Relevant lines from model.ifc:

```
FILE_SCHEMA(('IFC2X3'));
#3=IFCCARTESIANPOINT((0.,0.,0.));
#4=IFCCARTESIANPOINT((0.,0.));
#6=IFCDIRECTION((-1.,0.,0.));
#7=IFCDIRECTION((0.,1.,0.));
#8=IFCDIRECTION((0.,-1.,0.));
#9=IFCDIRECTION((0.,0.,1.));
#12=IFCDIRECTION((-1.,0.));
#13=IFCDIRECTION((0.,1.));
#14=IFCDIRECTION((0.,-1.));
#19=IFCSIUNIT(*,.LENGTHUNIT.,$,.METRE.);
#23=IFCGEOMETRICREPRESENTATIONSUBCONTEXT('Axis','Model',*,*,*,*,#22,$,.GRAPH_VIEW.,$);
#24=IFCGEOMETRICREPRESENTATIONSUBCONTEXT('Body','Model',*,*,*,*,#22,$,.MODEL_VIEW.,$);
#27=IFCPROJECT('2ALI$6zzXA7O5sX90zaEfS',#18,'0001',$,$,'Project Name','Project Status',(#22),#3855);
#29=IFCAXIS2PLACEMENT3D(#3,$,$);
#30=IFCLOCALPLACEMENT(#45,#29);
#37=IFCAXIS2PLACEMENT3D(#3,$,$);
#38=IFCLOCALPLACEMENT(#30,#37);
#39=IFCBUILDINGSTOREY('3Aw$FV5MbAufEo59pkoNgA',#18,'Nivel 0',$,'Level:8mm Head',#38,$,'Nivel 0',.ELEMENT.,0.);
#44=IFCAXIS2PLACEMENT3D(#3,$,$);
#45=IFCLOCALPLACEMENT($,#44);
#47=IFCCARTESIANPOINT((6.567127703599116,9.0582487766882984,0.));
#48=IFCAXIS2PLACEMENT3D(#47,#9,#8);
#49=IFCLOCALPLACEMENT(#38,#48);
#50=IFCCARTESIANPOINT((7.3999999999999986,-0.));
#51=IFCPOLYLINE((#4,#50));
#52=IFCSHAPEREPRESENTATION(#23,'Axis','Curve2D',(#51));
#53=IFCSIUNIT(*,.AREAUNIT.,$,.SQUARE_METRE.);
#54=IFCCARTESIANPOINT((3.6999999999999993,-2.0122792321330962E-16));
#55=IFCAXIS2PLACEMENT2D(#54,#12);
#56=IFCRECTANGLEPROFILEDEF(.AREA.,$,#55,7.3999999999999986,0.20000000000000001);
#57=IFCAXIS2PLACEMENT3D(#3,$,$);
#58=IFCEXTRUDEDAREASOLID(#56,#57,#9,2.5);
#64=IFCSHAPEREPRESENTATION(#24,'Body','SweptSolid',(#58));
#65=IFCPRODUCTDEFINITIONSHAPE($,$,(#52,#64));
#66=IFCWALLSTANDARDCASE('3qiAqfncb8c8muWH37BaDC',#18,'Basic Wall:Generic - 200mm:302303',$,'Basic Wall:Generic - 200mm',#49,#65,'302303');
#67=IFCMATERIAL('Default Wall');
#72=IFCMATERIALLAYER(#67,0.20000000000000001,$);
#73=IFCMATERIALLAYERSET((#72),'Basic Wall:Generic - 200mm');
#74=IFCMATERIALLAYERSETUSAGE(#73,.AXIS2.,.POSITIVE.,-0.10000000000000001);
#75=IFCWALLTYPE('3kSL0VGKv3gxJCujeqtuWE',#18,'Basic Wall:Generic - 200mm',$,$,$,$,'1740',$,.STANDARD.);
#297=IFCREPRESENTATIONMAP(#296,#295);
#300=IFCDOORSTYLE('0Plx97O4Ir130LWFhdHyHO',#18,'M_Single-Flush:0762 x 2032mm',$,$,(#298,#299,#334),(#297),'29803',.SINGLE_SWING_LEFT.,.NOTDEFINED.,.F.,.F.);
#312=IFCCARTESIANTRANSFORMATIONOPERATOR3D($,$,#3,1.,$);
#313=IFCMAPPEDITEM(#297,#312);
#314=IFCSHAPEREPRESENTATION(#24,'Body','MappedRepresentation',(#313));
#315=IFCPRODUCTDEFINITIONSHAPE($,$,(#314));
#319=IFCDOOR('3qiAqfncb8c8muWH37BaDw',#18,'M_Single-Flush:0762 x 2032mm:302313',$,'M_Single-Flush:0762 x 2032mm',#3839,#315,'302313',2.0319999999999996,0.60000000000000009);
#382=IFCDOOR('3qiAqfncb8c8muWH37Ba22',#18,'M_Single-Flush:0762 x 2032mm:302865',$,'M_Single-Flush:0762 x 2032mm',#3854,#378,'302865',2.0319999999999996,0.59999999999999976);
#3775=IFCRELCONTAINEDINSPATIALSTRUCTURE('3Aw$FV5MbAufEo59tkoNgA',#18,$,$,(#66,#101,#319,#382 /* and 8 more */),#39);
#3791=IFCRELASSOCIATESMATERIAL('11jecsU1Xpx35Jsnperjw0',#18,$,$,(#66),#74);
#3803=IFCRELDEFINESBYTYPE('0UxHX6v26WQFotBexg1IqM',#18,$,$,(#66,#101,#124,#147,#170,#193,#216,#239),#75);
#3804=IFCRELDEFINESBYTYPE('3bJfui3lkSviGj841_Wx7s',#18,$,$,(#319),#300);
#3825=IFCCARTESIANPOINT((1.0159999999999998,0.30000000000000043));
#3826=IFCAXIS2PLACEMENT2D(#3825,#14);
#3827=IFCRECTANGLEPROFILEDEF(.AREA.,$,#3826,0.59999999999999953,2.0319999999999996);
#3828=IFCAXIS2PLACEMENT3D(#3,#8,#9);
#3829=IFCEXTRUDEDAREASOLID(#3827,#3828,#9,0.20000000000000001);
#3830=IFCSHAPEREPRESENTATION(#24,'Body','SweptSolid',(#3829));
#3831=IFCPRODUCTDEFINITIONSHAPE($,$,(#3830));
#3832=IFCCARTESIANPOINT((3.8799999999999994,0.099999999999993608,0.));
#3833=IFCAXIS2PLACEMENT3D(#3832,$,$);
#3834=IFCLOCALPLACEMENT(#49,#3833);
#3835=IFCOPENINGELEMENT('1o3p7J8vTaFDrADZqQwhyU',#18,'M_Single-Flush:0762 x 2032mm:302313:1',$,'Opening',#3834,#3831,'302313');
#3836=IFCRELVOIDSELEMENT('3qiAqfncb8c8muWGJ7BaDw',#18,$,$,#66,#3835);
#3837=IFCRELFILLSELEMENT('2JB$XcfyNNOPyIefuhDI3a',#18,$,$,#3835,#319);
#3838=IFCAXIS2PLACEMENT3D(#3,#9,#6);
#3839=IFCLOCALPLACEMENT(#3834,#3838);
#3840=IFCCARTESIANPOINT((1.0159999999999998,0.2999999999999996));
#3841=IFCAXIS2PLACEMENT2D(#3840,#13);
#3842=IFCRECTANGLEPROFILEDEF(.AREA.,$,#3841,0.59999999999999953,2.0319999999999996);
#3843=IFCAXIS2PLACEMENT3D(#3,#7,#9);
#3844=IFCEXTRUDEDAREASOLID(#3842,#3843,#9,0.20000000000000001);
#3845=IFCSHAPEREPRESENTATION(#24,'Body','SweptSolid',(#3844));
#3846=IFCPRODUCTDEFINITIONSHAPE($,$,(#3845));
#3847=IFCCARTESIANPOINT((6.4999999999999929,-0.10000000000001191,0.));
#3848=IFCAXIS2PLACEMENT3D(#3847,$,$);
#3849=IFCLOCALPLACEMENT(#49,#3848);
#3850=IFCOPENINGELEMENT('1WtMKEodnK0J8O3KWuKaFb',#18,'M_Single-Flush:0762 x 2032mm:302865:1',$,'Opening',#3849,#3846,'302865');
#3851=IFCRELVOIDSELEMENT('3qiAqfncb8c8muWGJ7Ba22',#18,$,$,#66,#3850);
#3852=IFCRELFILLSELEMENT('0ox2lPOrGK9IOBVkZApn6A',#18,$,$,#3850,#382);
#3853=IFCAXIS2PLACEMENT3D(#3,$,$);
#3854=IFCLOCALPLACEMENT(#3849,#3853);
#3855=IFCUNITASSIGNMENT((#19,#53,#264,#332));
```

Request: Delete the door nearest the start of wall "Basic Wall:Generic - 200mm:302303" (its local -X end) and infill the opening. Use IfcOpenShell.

```python
import ifcopenshell
import ifcopenshell.api.feature
import ifcopenshell.api.root
import ifcopenshell.geom
import ifcopenshell.util.shape

model = ifcopenshell.open("model.ifc")
settings = ifcopenshell.geom.settings()


def volume(element):
    """Net volume in cubic metres, openings subtracted."""
    shape = ifcopenshell.geom.create_shape(settings, element)
    return ifcopenshell.util.shape.get_volume(shape.geometry)


door = model.by_guid("3qiAqfncb8c8muWH37BaDw")
opening = door.FillsVoids[0].RelatingOpeningElement
wall = opening.VoidsElements[0].RelatingBuildingElement
before = volume(wall)

ifcopenshell.api.root.remove_product(model, product=door)
ifcopenshell.api.feature.remove_feature(model, feature=opening)

after = volume(wall)

print(f"wall volume {before:.3f} -> {after:.3f} m3")

model.write("model_updated.ifc")
```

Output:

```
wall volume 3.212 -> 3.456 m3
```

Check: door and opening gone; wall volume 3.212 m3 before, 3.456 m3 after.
